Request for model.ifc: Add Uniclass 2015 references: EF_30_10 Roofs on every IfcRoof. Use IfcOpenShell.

First a look at what the model holds.

```python
import ifcopenshell

model = ifcopenshell.open("model.ifc")
print(model.schema)
print("classifications:", [c.Name for c in model.by_type("IfcClassification")])
for ifc_class in ("IfcDoor", "IfcRoof", "IfcStair", "IfcWall", "IfcWindow"):
    print(ifc_class, len(model.by_type(ifc_class)))
```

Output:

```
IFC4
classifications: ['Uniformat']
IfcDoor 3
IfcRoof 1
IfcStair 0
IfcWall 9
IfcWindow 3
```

```python
import ifcopenshell
import ifcopenshell.api.classification

model = ifcopenshell.open("model.ifc")

system = ifcopenshell.api.classification.add_classification(model, classification="Uniclass 2015")

codes = {
    "IfcRoof": ("EF_30_10", "Roofs"),
}
for ifc_class, (code, name) in codes.items():
    products = model.by_type(ifc_class)
    ifcopenshell.api.classification.add_reference(
        model, products=products, classification=system, identification=code, name=name
    )
    print(code, len(products))

model.write("model_edited.ifc")
```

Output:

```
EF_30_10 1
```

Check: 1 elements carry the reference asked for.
